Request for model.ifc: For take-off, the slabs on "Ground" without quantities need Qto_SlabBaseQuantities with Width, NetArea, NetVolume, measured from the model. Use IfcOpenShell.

First a look at what the model holds.

```python
import ifcopenshell
import ifcopenshell.util.element
import ifcopenshell.util.unit

model = ifcopenshell.open("model.ifc")
print(model.schema)
for unit_type in ("LENGTHUNIT", "AREAUNIT", "VOLUMEUNIT"):
    print(unit_type, ifcopenshell.util.unit.calculate_unit_scale(model, unit_type))
storey = next(s for s in model.by_type("IfcBuildingStorey") if s.Name == "Ground")
slabs = [e for e in ifcopenshell.util.element.get_decomposition(storey) if e.is_a("IfcSlab")]
for e in sorted(slabs, key=lambda e: e.id()):
    print(e.id(), e.is_a(), e.Name, list(ifcopenshell.util.element.get_psets(e, qtos_only=True)), sep=" | ")
```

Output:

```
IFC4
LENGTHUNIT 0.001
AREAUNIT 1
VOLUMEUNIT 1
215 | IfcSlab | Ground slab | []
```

```python
import ifcopenshell
import ifcopenshell.api.pset
import ifcopenshell.geom
import ifcopenshell.util.element
import ifcopenshell.util.shape
import ifcopenshell.util.unit

model = ifcopenshell.open("model.ifc")
unit_scale = ifcopenshell.util.unit.calculate_unit_scale(model)
area_scale = ifcopenshell.util.unit.calculate_unit_scale(model, "AREAUNIT")
volume_scale = ifcopenshell.util.unit.calculate_unit_scale(model, "VOLUMEUNIT")
settings = ifcopenshell.geom.settings()

storey = next(s for s in model.by_type("IfcBuildingStorey") if s.Name == "Ground")
slabs = [e for e in ifcopenshell.util.element.get_decomposition(storey) if e.is_a("IfcSlab")]

for e in sorted(slabs, key=lambda e: e.id()):
    if ifcopenshell.util.element.get_psets(e, qtos_only=True, should_inherit=False):
        continue
    # Geometry comes back in metres, in the element's own axes.
    shape = ifcopenshell.geom.create_shape(settings, e)
    values = {
        "Width": ifcopenshell.util.shape.get_z(shape.geometry) / unit_scale,
        "NetArea": ifcopenshell.util.shape.get_footprint_area(shape.geometry) / area_scale,
        "NetVolume": ifcopenshell.util.shape.get_volume(shape.geometry) / volume_scale,
    }
    qto = ifcopenshell.api.pset.add_qto(model, product=e, name="Qto_SlabBaseQuantities")
    ifcopenshell.api.pset.edit_qto(model, qto=qto, properties=values)
    print(e.id(), {k: round(v, 3) for k, v in values.items()})

model.write("model_rev.ifc")
```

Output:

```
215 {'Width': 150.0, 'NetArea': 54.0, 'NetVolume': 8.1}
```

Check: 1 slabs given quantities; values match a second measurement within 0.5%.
